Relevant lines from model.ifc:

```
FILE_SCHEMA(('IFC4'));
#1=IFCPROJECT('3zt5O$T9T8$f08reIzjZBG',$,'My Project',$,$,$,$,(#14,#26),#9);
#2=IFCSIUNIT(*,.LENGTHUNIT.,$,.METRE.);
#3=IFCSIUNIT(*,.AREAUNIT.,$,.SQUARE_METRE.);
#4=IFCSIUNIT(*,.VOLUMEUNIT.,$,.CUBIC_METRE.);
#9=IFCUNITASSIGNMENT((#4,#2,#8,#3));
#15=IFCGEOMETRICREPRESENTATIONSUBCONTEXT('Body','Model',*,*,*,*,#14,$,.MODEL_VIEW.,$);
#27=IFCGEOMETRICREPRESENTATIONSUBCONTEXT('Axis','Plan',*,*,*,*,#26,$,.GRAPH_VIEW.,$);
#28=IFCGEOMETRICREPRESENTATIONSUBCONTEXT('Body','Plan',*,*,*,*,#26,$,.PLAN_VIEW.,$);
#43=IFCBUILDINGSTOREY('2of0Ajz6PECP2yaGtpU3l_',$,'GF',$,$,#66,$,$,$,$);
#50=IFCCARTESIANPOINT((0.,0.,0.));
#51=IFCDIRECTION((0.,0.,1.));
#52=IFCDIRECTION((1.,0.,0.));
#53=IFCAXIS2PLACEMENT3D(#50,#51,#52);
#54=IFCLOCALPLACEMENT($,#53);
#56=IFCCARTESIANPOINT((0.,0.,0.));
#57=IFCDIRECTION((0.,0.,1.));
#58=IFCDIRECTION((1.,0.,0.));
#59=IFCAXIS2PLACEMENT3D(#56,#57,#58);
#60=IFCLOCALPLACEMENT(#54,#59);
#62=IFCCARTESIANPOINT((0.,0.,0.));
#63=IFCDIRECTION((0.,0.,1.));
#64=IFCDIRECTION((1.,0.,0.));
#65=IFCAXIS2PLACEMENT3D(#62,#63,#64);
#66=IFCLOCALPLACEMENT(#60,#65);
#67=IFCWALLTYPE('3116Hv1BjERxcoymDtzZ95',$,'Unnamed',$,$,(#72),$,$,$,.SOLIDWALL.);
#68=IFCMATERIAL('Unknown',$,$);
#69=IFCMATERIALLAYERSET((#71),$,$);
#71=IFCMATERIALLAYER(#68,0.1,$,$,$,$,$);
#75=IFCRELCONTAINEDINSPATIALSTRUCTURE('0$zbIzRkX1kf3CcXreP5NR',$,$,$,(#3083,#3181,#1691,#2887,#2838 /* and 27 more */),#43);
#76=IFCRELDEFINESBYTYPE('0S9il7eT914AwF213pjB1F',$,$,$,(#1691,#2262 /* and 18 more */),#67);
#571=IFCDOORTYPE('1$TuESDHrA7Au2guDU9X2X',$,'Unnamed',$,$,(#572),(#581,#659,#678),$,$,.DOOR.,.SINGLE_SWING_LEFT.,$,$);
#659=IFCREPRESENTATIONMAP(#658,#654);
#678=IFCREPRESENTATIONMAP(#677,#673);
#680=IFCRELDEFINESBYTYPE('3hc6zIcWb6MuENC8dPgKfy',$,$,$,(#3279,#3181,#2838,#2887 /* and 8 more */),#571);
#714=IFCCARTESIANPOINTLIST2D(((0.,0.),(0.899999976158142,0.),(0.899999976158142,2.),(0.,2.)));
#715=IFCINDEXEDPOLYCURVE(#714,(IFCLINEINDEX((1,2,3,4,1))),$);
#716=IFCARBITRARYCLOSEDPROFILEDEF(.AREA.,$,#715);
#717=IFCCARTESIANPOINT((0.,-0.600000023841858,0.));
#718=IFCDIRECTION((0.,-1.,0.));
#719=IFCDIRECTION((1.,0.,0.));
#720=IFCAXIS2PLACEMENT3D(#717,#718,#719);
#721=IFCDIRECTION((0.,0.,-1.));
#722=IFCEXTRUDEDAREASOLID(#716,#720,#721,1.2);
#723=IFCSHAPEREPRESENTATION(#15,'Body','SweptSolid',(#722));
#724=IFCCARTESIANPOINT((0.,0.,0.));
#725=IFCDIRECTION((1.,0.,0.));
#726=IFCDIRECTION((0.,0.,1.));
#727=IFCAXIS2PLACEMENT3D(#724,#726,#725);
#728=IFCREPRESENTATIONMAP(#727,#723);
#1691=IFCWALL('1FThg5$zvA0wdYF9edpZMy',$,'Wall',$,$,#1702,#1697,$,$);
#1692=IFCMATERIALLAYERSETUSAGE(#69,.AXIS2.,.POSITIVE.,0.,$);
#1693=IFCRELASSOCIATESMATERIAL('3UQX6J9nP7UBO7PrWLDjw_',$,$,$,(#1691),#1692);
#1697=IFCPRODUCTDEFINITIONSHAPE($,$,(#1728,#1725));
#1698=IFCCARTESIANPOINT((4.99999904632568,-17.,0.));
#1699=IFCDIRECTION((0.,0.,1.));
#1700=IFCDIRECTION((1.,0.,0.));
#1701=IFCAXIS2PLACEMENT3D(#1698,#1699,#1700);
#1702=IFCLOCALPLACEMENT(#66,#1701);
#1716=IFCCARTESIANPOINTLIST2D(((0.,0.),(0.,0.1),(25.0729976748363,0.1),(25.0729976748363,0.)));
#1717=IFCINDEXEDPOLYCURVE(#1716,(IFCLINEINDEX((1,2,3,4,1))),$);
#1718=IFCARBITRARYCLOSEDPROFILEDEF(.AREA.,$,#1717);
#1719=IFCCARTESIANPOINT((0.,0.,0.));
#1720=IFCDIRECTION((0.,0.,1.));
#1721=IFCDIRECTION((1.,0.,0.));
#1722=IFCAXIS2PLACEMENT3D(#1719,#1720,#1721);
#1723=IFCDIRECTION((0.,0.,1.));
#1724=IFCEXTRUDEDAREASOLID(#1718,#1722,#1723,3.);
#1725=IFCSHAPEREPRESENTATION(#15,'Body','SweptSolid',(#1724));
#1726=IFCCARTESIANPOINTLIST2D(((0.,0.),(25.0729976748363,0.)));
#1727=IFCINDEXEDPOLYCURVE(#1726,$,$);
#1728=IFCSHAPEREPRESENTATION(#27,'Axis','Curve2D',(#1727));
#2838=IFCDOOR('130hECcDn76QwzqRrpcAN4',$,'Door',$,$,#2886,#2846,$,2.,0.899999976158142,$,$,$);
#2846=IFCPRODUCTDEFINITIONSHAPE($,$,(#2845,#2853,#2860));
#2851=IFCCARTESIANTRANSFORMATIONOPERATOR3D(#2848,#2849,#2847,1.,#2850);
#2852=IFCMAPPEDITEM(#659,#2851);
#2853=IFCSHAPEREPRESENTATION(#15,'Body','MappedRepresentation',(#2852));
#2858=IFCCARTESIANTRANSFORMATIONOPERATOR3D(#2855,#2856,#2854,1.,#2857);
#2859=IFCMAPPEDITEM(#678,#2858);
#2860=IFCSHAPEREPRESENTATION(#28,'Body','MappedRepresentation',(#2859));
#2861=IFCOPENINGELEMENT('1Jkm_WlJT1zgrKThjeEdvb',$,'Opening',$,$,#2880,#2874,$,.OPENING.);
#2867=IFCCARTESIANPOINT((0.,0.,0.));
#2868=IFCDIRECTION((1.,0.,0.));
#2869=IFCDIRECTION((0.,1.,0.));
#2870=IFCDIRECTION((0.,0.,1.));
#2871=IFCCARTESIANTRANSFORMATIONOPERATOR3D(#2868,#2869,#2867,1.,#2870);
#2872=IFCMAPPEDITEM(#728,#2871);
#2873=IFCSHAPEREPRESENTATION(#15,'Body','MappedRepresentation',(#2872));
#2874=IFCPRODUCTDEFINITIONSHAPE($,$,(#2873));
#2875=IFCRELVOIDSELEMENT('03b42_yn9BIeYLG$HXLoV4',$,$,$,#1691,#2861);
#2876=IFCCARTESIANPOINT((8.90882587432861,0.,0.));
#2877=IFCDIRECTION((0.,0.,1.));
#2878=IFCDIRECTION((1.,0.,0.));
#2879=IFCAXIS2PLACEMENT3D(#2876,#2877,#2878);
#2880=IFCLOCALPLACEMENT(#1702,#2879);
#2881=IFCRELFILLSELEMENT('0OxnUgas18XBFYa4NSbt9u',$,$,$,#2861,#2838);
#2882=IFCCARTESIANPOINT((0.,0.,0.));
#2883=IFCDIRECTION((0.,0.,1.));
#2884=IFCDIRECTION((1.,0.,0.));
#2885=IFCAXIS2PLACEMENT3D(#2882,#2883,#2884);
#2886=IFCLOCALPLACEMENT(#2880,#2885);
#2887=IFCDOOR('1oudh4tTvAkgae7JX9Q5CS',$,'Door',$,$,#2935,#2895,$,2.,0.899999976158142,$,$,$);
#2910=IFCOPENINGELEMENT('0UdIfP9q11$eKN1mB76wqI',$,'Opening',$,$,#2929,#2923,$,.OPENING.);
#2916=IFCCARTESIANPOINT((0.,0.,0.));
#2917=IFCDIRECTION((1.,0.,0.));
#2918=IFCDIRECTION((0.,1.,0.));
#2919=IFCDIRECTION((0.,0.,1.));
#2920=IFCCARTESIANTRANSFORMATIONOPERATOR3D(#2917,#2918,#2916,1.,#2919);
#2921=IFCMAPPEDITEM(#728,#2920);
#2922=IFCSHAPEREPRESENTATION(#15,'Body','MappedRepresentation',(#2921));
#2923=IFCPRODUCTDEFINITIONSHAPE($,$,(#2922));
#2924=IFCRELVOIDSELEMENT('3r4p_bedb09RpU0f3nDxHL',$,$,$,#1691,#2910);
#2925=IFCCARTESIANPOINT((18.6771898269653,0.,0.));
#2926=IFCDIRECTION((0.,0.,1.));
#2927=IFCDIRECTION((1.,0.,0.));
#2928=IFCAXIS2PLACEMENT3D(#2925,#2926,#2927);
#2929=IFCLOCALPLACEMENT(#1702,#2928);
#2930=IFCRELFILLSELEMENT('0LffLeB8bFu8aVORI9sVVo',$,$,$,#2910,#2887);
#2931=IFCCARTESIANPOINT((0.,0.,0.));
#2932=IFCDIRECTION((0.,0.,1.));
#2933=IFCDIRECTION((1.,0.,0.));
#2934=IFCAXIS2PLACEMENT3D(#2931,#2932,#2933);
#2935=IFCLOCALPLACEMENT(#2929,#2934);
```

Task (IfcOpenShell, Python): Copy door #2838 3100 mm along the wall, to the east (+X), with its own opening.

```python
import ifcopenshell
import ifcopenshell.api.feature
import ifcopenshell.api.geometry
import ifcopenshell.api.root
import ifcopenshell.geom
import ifcopenshell.util.element
import ifcopenshell.util.placement
import ifcopenshell.util.shape
import ifcopenshell.util.unit

model = ifcopenshell.open("model.ifc")
unit_scale = ifcopenshell.util.unit.calculate_unit_scale(model)
settings = ifcopenshell.geom.settings()


def volume(element):
    """Net volume in cubic metres, openings subtracted."""
    shape = ifcopenshell.geom.create_shape(settings, element)
    return ifcopenshell.util.shape.get_volume(shape.geometry)


door = model.by_id(2838)
opening = door.FillsVoids[0].RelatingOpeningElement
wall = opening.VoidsElements[0].RelatingBuildingElement
before = volume(wall)
shift = ifcopenshell.util.placement.get_local_placement(wall.ObjectPlacement)[:3, 0] * 3.1 / unit_scale

# copy_class copies the void relationship, type, container and properties, but no geometry.
new_opening = ifcopenshell.api.root.copy_class(model, product=opening)
new_opening.Representation = ifcopenshell.util.element.copy_deep(
    model, opening.Representation, exclude=["IfcGeometricRepresentationContext", "IfcRepresentationMap"]
)
new_door = ifcopenshell.api.root.copy_class(model, product=door)
new_door.Representation = ifcopenshell.util.element.copy_deep(
    model, door.Representation, exclude=["IfcGeometricRepresentationContext", "IfcRepresentationMap"]
)
ifcopenshell.api.feature.add_filling(model, opening=new_opening, element=new_door)

for old, new in ((opening, new_opening), (door, new_door)):
    matrix = ifcopenshell.util.placement.get_local_placement(old.ObjectPlacement)
    matrix[:3, 3] += shift
    ifcopenshell.api.geometry.edit_object_placement(model, product=new, matrix=matrix, is_si=False)

after = volume(wall)

print(f"wall volume {before:.3f} -> {after:.3f} m3")

model.write("model_updated.ifc")
```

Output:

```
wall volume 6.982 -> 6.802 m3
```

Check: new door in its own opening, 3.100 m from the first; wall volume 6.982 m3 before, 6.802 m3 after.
